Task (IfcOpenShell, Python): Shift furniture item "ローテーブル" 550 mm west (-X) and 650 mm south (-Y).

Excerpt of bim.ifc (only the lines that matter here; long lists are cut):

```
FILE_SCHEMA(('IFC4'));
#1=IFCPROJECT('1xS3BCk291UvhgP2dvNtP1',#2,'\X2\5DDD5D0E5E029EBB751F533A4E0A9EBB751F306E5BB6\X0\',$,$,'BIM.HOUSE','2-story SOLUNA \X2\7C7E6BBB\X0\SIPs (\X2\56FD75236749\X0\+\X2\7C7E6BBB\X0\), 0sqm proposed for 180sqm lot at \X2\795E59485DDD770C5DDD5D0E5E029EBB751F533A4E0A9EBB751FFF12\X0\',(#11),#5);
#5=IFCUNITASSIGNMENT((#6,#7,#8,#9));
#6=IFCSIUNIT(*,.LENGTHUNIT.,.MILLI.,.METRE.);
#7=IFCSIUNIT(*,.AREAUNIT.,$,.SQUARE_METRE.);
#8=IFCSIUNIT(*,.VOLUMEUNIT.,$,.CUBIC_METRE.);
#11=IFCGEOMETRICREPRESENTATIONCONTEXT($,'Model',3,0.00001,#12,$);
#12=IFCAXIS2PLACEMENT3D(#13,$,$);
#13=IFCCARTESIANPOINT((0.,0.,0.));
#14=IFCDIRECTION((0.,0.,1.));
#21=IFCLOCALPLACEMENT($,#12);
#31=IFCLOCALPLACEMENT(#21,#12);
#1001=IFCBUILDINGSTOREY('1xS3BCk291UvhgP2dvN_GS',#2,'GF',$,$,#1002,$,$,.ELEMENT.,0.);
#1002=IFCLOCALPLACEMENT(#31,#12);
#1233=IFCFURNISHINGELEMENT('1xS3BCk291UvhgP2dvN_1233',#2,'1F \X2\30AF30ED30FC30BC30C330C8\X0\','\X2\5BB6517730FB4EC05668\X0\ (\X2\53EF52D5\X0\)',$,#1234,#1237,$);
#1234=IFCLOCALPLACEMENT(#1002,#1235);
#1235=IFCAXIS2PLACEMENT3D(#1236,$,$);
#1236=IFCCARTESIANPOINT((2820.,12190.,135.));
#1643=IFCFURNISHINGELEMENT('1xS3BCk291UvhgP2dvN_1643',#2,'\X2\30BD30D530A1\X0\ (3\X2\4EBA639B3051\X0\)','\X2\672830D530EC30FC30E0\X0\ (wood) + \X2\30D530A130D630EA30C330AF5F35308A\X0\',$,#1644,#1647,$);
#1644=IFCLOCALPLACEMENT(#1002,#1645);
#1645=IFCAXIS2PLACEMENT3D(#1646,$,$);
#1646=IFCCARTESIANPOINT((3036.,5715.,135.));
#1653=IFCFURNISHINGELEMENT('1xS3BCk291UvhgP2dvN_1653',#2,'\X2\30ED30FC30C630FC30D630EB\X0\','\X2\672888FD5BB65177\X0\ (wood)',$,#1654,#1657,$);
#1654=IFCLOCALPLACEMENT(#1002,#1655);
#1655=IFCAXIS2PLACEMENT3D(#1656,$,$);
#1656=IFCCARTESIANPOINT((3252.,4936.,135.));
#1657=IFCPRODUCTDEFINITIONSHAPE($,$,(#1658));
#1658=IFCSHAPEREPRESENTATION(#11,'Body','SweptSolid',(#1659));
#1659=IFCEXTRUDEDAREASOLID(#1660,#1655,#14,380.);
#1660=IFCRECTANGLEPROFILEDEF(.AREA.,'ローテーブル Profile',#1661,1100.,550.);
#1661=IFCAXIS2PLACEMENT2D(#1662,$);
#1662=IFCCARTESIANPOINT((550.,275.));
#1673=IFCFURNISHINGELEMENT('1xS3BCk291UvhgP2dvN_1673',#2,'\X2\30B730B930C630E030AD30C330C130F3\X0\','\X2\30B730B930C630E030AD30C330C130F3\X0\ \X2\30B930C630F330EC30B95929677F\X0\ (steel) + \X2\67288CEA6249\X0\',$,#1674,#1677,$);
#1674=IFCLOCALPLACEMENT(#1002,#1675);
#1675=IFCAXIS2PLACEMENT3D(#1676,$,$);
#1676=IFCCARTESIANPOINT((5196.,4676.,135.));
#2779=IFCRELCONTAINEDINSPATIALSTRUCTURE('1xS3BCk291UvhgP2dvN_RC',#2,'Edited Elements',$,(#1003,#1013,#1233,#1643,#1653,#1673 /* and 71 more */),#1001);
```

```python
import ifcopenshell
import ifcopenshell.api.geometry
import ifcopenshell.util.placement
import ifcopenshell.util.unit

model = ifcopenshell.open("bim.ifc")
unit_scale = ifcopenshell.util.unit.calculate_unit_scale(model)

item = model.by_id(1653)
matrix = ifcopenshell.util.placement.get_local_placement(item.ObjectPlacement)
matrix[0, 3] -= 0.55 / unit_scale
matrix[1, 3] -= 0.65 / unit_scale
ifcopenshell.api.geometry.edit_object_placement(model, product=item, matrix=matrix, is_si=False)

print(ifcopenshell.util.placement.get_local_placement(item.ObjectPlacement).round(3) + 0.0)

model.write("bim_rev.ifc")
```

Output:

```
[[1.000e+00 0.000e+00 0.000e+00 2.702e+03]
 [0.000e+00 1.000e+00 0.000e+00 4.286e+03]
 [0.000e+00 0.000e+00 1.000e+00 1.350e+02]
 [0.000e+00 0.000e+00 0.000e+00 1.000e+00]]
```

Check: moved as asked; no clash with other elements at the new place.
